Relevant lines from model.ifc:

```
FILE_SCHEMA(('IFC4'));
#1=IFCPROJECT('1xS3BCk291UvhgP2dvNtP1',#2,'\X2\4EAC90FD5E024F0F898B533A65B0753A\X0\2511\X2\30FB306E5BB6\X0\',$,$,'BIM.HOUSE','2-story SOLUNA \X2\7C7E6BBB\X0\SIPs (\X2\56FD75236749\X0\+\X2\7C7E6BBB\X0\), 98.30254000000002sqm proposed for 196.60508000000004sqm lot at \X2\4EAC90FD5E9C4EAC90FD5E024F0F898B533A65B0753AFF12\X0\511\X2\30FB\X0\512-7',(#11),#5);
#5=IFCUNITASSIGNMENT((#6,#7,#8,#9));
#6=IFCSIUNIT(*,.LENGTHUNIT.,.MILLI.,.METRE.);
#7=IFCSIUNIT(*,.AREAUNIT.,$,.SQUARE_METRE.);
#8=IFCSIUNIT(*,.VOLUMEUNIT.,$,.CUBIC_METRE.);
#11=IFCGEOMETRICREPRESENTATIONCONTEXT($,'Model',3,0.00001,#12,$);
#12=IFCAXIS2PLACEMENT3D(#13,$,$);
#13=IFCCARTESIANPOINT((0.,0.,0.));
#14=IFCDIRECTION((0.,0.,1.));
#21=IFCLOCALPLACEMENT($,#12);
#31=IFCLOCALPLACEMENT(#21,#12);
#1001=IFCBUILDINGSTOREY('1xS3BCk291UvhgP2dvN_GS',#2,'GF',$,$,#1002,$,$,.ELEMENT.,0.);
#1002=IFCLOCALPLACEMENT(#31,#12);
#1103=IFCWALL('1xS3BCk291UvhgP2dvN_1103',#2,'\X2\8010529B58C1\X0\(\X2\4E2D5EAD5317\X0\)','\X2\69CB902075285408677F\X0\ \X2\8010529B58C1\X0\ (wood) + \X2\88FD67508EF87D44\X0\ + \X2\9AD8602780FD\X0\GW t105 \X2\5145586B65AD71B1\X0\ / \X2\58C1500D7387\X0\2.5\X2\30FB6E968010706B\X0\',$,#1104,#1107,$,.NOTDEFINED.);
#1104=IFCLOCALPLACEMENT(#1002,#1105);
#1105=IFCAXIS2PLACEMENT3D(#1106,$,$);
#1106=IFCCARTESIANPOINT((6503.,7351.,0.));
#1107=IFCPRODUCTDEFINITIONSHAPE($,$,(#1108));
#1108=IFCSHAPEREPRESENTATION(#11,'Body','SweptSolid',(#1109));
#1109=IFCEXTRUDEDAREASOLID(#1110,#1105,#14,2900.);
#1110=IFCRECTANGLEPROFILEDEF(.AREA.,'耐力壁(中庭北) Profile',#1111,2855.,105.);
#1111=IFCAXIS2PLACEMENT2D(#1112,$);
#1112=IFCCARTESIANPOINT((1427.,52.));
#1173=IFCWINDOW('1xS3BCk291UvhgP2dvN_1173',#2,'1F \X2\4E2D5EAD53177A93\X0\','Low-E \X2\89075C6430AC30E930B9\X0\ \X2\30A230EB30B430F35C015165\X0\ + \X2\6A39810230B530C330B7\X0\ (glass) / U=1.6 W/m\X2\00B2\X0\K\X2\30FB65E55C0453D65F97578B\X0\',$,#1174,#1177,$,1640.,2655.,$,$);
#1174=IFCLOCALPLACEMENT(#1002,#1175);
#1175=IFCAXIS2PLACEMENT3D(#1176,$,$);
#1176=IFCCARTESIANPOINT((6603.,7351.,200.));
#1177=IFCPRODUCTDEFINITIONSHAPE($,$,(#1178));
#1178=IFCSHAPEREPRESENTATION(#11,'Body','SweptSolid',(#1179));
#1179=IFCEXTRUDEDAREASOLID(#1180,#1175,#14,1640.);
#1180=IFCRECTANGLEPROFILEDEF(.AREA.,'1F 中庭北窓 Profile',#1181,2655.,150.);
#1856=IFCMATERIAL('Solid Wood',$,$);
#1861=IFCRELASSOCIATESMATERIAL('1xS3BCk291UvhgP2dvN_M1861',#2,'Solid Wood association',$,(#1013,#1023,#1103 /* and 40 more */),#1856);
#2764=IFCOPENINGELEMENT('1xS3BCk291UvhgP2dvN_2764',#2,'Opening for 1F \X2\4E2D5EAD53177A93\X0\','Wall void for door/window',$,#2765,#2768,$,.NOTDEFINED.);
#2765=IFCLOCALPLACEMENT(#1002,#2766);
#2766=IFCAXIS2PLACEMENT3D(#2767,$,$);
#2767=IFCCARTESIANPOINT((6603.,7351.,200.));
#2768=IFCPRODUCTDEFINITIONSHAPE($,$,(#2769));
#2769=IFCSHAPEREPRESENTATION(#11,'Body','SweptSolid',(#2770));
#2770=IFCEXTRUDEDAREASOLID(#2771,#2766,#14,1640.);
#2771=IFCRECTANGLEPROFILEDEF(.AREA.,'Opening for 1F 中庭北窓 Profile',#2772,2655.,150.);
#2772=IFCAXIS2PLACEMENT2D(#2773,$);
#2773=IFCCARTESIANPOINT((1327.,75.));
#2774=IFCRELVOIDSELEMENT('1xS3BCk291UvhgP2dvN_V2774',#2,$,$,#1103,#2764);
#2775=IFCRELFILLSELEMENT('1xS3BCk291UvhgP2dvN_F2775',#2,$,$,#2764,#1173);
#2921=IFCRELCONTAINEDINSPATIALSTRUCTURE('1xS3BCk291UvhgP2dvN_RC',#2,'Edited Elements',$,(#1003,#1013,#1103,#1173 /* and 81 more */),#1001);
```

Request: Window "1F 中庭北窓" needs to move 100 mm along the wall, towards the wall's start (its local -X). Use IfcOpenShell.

```python
import ifcopenshell
import ifcopenshell.api.geometry
import ifcopenshell.util.placement

model = ifcopenshell.open("model.ifc")

window = model.by_guid("1xS3BCk291UvhgP2dvN_1173")
opening = window.FillsVoids[0].RelatingOpeningElement
wall = opening.VoidsElements[0].RelatingBuildingElement

wall_matrix = ifcopenshell.util.placement.get_local_placement(wall.ObjectPlacement)
shift = wall_matrix[:3, 0] * -100.0
before = ifcopenshell.util.placement.get_local_placement(window.ObjectPlacement)[:3, 3].copy()

# The window is not placed relative to its opening, so move both.
for product in (opening, window):
    matrix = ifcopenshell.util.placement.get_local_placement(product.ObjectPlacement)
    matrix[:3, 3] += shift
    ifcopenshell.api.geometry.edit_object_placement(model, product=product, matrix=matrix, is_si=False)

after = ifcopenshell.util.placement.get_local_placement(window.ObjectPlacement)[:3, 3]
print("window moved by", (after - before).round(3) + 0.0)

model.write("model_v2.ifc")
```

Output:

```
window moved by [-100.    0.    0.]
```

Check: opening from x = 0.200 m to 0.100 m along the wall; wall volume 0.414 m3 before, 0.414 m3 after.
